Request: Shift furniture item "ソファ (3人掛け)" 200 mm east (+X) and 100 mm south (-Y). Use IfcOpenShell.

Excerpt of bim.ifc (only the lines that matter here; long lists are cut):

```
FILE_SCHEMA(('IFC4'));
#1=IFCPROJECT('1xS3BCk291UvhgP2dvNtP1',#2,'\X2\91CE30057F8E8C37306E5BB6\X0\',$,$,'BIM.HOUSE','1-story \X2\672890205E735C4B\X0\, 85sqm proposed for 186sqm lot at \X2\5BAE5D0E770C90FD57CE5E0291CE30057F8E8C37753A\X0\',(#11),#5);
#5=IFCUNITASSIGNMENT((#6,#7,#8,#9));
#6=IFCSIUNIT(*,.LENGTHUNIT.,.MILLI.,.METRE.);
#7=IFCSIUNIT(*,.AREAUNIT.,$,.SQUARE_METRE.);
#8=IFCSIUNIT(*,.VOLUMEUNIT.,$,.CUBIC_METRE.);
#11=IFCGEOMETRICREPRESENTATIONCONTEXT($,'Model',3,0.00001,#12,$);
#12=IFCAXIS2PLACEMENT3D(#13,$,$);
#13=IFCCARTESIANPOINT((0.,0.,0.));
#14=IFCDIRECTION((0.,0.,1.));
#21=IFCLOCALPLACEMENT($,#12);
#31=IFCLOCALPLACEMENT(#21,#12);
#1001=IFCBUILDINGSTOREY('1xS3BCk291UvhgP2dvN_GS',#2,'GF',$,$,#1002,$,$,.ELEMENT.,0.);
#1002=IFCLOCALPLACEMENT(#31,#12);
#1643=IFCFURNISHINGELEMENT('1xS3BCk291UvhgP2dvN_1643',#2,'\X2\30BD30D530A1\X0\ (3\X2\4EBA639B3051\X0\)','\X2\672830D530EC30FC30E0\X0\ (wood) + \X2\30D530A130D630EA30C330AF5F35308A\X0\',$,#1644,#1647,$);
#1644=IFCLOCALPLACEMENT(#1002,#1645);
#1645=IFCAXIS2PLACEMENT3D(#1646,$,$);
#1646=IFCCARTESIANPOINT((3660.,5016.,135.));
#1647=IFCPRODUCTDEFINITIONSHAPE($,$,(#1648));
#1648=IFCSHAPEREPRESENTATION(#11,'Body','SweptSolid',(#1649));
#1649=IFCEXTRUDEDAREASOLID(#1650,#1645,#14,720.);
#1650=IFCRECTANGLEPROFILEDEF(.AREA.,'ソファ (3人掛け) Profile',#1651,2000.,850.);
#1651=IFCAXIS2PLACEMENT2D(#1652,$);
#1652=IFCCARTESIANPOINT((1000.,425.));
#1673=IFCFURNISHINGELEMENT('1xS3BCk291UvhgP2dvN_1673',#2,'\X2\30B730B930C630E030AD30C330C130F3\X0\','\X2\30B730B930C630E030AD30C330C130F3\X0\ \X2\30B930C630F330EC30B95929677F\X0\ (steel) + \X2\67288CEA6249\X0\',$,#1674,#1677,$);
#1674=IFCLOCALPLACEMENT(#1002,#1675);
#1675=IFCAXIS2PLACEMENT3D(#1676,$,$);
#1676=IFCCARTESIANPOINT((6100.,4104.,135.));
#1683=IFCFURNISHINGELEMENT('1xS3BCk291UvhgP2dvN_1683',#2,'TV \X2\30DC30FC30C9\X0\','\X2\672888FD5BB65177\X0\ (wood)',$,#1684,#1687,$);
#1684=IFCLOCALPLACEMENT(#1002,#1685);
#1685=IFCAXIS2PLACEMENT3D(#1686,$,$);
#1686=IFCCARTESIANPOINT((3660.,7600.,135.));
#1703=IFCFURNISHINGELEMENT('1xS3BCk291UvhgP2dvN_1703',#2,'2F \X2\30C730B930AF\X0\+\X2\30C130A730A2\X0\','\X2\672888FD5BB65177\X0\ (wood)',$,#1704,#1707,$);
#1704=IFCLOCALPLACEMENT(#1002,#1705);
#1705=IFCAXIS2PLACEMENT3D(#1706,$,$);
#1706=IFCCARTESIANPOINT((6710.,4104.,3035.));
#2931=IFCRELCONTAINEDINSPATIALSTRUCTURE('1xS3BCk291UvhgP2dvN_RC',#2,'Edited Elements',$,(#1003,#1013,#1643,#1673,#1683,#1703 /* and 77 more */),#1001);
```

```python
import ifcopenshell
import ifcopenshell.api.geometry
import ifcopenshell.util.placement
import ifcopenshell.util.unit

model = ifcopenshell.open("bim.ifc")
unit_scale = ifcopenshell.util.unit.calculate_unit_scale(model)

item = model.by_id(1643)
matrix = ifcopenshell.util.placement.get_local_placement(item.ObjectPlacement)
matrix[0, 3] += 0.2 / unit_scale
matrix[1, 3] -= 0.1 / unit_scale
ifcopenshell.api.geometry.edit_object_placement(model, product=item, matrix=matrix, is_si=False)

print(ifcopenshell.util.placement.get_local_placement(item.ObjectPlacement).round(3) + 0.0)

model.write("bim_updated.ifc")
```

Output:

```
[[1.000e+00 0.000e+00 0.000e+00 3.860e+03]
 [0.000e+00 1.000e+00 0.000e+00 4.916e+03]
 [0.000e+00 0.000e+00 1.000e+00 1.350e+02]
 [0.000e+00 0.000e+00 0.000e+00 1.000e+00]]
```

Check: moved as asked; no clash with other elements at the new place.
